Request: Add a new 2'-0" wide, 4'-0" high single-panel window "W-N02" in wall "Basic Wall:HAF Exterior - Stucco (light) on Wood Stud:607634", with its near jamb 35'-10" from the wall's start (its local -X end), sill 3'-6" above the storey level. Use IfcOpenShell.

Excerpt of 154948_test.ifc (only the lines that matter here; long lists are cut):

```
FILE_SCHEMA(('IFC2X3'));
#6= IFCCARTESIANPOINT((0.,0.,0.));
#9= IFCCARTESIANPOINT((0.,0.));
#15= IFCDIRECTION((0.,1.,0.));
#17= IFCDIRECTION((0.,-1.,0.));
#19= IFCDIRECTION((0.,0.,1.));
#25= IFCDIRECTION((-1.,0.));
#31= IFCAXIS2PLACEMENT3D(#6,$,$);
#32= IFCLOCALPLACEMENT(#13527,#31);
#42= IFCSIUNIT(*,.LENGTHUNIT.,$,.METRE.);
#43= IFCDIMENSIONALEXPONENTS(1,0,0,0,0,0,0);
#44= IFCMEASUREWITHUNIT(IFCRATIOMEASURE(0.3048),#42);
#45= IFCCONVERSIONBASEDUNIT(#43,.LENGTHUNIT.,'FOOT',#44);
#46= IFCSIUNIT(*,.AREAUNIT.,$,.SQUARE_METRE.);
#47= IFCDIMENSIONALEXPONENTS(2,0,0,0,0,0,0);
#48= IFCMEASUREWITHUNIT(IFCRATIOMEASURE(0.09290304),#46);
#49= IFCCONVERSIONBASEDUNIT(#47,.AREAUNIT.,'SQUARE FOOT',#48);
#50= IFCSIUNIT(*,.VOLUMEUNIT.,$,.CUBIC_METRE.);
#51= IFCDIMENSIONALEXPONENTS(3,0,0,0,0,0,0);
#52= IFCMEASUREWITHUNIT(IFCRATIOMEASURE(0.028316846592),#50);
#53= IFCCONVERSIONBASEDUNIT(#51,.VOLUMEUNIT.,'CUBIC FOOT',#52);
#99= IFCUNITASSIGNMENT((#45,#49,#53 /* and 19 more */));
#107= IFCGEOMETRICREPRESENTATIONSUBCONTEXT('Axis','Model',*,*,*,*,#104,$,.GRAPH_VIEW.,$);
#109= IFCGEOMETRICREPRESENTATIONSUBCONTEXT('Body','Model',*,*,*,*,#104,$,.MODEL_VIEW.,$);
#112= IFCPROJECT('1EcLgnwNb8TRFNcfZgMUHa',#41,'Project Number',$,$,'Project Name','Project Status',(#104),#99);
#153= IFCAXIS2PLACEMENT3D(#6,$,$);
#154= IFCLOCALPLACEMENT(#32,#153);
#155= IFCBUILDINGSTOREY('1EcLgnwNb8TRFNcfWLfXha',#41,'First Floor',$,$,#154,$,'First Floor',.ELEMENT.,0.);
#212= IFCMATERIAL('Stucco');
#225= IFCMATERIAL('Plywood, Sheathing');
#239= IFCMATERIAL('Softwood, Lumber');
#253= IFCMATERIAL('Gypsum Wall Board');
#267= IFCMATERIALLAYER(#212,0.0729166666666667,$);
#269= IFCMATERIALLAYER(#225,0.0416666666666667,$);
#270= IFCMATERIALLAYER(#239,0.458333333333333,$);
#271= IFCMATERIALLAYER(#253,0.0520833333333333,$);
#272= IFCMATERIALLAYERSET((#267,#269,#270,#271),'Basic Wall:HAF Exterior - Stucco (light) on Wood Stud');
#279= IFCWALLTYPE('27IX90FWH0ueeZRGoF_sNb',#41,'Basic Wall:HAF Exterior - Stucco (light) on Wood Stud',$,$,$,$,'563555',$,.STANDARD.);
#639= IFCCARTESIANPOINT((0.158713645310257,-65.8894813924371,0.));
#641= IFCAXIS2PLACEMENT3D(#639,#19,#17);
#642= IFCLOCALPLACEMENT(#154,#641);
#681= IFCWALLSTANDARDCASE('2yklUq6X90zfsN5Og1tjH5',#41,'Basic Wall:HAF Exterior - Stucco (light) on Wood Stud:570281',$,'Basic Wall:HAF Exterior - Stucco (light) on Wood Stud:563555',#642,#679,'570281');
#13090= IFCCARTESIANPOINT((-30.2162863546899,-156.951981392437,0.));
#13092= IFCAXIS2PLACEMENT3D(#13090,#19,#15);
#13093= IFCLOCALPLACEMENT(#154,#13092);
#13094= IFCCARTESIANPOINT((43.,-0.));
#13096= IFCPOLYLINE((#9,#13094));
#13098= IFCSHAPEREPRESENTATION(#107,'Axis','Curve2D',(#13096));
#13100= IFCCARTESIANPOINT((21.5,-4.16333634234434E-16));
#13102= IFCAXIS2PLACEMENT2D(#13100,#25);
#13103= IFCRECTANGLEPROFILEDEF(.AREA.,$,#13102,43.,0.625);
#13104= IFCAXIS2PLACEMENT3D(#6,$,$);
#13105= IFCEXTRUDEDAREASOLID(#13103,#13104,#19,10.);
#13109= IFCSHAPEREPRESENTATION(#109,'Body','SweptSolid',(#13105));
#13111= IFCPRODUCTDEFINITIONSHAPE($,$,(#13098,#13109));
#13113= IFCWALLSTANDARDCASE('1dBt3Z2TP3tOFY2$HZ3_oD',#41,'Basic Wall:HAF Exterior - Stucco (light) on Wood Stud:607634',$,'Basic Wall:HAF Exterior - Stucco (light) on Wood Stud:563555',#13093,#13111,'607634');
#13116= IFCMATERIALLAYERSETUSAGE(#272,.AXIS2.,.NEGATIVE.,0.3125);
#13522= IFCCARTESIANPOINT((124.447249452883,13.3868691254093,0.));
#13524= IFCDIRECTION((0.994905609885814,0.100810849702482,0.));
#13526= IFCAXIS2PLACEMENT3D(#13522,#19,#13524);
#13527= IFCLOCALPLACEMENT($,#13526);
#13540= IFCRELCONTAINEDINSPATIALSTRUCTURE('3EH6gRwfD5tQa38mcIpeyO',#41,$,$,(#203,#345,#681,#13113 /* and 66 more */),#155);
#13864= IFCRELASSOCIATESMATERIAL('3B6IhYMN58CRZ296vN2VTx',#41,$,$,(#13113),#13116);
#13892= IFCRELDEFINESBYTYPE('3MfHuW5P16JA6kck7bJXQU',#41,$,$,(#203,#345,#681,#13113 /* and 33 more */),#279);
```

```python
import numpy as np
import ifcopenshell
import ifcopenshell.api.feature
import ifcopenshell.api.geometry
import ifcopenshell.api.root
import ifcopenshell.api.spatial
import ifcopenshell.api.type
import ifcopenshell.geom
import ifcopenshell.util.element
import ifcopenshell.util.placement
import ifcopenshell.util.representation
import ifcopenshell.util.shape
import ifcopenshell.util.unit

model = ifcopenshell.open("154948_test.ifc")
unit_scale = ifcopenshell.util.unit.calculate_unit_scale(model)
settings = ifcopenshell.geom.settings()


def volume(element):
    """Net volume in cubic metres, openings subtracted."""
    shape = ifcopenshell.geom.create_shape(settings, element)
    return ifcopenshell.util.shape.get_volume(shape.geometry)


wall = model.by_id(13113)
storey = ifcopenshell.util.element.get_container(wall, ifc_class="IfcBuildingStorey")
context = ifcopenshell.util.representation.get_context(model, "Model", "Body", "MODEL_VIEW")
before = volume(wall)

width, height, from_end, sill = 0.6096, 1.2192, 10.922, 1.0668  # metres

# The wall runs along its own X axis, and the end named is its -X end.
wall_shape = ifcopenshell.geom.create_shape(settings, wall)
x, y, z = ifcopenshell.util.shape.get_vertices(wall_shape.geometry).T
start = x.min() + from_end
face, thickness = float(y.min()), float(y.max() - y.min())
wall_matrix = ifcopenshell.util.placement.get_local_placement(wall.ObjectPlacement)
level = ifcopenshell.util.placement.get_local_placement(storey.ObjectPlacement)[2, 3]


def in_wall(x, y):
    """Placement at x, y metres in the wall's axes, at sill height."""
    matrix = wall_matrix.copy()
    matrix[:, 3] = wall_matrix @ np.array([x / unit_scale, y / unit_scale, 0.0, 1.0])
    matrix[2, 3] = level + sill / unit_scale
    return matrix


# Opening: a box that overshoots both wall faces by 50 mm.
opening = ifcopenshell.api.root.create_entity(model, ifc_class="IfcOpeningElement")
box = ifcopenshell.api.geometry.add_wall_representation(
    model, context=context, length=width, height=height, thickness=thickness + 0.1
)
ifcopenshell.api.geometry.assign_representation(model, product=opening, representation=box)
ifcopenshell.api.geometry.edit_object_placement(model, product=opening, matrix=in_wall(start, face - 0.05), is_si=False)
ifcopenshell.api.feature.add_feature(model, feature=opening, element=wall)

window = ifcopenshell.api.root.create_entity(model, ifc_class="IfcWindow", name="W-N02")
window.OverallWidth, window.OverallHeight = width / unit_scale, height / unit_scale
body = ifcopenshell.api.geometry.add_window_representation(
    model,
    context=context,
    overall_width=window.OverallWidth,
    overall_height=window.OverallHeight,
    partition_type="SINGLE_PANEL",
)
ifcopenshell.api.geometry.assign_representation(model, product=window, representation=body)
ifcopenshell.api.spatial.assign_container(model, products=[window], relating_structure=storey)
fills = ifcopenshell.api.feature.add_filling(model, opening=opening, element=window)
fills.OwnerHistory = window.OwnerHistory  # required in IFC2X3

# IFC2X3 keeps the operation on the window style.
style = ifcopenshell.api.root.create_entity(model, ifc_class="IfcWindowStyle", name="W-N02")
style.OperationType, style.ConstructionType = "SINGLE_PANEL", "NOTDEFINED"
style.ParameterTakesPrecedence = style.Sizeable = False
ifcopenshell.api.type.assign_type(model, related_objects=[window], relating_type=style)

# Centre the window in the wall's thickness.
ifcopenshell.api.geometry.edit_object_placement(model, product=window, matrix=in_wall(start, face), is_si=False)
window_shape = ifcopenshell.geom.create_shape(settings, window)
depth = ifcopenshell.util.shape.get_vertices(window_shape.geometry)[:, 1]
offset = face + thickness / 2 - (depth.min() + depth.max()) / 2
ifcopenshell.api.geometry.edit_object_placement(model, product=window, matrix=in_wall(start, offset), is_si=False)

after = volume(wall)

print(f"wall volume {before:.3f} -> {after:.3f} m3")

model.write("154948_test_rev.ifc")
```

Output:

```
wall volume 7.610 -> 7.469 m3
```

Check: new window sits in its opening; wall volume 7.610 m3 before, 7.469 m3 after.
